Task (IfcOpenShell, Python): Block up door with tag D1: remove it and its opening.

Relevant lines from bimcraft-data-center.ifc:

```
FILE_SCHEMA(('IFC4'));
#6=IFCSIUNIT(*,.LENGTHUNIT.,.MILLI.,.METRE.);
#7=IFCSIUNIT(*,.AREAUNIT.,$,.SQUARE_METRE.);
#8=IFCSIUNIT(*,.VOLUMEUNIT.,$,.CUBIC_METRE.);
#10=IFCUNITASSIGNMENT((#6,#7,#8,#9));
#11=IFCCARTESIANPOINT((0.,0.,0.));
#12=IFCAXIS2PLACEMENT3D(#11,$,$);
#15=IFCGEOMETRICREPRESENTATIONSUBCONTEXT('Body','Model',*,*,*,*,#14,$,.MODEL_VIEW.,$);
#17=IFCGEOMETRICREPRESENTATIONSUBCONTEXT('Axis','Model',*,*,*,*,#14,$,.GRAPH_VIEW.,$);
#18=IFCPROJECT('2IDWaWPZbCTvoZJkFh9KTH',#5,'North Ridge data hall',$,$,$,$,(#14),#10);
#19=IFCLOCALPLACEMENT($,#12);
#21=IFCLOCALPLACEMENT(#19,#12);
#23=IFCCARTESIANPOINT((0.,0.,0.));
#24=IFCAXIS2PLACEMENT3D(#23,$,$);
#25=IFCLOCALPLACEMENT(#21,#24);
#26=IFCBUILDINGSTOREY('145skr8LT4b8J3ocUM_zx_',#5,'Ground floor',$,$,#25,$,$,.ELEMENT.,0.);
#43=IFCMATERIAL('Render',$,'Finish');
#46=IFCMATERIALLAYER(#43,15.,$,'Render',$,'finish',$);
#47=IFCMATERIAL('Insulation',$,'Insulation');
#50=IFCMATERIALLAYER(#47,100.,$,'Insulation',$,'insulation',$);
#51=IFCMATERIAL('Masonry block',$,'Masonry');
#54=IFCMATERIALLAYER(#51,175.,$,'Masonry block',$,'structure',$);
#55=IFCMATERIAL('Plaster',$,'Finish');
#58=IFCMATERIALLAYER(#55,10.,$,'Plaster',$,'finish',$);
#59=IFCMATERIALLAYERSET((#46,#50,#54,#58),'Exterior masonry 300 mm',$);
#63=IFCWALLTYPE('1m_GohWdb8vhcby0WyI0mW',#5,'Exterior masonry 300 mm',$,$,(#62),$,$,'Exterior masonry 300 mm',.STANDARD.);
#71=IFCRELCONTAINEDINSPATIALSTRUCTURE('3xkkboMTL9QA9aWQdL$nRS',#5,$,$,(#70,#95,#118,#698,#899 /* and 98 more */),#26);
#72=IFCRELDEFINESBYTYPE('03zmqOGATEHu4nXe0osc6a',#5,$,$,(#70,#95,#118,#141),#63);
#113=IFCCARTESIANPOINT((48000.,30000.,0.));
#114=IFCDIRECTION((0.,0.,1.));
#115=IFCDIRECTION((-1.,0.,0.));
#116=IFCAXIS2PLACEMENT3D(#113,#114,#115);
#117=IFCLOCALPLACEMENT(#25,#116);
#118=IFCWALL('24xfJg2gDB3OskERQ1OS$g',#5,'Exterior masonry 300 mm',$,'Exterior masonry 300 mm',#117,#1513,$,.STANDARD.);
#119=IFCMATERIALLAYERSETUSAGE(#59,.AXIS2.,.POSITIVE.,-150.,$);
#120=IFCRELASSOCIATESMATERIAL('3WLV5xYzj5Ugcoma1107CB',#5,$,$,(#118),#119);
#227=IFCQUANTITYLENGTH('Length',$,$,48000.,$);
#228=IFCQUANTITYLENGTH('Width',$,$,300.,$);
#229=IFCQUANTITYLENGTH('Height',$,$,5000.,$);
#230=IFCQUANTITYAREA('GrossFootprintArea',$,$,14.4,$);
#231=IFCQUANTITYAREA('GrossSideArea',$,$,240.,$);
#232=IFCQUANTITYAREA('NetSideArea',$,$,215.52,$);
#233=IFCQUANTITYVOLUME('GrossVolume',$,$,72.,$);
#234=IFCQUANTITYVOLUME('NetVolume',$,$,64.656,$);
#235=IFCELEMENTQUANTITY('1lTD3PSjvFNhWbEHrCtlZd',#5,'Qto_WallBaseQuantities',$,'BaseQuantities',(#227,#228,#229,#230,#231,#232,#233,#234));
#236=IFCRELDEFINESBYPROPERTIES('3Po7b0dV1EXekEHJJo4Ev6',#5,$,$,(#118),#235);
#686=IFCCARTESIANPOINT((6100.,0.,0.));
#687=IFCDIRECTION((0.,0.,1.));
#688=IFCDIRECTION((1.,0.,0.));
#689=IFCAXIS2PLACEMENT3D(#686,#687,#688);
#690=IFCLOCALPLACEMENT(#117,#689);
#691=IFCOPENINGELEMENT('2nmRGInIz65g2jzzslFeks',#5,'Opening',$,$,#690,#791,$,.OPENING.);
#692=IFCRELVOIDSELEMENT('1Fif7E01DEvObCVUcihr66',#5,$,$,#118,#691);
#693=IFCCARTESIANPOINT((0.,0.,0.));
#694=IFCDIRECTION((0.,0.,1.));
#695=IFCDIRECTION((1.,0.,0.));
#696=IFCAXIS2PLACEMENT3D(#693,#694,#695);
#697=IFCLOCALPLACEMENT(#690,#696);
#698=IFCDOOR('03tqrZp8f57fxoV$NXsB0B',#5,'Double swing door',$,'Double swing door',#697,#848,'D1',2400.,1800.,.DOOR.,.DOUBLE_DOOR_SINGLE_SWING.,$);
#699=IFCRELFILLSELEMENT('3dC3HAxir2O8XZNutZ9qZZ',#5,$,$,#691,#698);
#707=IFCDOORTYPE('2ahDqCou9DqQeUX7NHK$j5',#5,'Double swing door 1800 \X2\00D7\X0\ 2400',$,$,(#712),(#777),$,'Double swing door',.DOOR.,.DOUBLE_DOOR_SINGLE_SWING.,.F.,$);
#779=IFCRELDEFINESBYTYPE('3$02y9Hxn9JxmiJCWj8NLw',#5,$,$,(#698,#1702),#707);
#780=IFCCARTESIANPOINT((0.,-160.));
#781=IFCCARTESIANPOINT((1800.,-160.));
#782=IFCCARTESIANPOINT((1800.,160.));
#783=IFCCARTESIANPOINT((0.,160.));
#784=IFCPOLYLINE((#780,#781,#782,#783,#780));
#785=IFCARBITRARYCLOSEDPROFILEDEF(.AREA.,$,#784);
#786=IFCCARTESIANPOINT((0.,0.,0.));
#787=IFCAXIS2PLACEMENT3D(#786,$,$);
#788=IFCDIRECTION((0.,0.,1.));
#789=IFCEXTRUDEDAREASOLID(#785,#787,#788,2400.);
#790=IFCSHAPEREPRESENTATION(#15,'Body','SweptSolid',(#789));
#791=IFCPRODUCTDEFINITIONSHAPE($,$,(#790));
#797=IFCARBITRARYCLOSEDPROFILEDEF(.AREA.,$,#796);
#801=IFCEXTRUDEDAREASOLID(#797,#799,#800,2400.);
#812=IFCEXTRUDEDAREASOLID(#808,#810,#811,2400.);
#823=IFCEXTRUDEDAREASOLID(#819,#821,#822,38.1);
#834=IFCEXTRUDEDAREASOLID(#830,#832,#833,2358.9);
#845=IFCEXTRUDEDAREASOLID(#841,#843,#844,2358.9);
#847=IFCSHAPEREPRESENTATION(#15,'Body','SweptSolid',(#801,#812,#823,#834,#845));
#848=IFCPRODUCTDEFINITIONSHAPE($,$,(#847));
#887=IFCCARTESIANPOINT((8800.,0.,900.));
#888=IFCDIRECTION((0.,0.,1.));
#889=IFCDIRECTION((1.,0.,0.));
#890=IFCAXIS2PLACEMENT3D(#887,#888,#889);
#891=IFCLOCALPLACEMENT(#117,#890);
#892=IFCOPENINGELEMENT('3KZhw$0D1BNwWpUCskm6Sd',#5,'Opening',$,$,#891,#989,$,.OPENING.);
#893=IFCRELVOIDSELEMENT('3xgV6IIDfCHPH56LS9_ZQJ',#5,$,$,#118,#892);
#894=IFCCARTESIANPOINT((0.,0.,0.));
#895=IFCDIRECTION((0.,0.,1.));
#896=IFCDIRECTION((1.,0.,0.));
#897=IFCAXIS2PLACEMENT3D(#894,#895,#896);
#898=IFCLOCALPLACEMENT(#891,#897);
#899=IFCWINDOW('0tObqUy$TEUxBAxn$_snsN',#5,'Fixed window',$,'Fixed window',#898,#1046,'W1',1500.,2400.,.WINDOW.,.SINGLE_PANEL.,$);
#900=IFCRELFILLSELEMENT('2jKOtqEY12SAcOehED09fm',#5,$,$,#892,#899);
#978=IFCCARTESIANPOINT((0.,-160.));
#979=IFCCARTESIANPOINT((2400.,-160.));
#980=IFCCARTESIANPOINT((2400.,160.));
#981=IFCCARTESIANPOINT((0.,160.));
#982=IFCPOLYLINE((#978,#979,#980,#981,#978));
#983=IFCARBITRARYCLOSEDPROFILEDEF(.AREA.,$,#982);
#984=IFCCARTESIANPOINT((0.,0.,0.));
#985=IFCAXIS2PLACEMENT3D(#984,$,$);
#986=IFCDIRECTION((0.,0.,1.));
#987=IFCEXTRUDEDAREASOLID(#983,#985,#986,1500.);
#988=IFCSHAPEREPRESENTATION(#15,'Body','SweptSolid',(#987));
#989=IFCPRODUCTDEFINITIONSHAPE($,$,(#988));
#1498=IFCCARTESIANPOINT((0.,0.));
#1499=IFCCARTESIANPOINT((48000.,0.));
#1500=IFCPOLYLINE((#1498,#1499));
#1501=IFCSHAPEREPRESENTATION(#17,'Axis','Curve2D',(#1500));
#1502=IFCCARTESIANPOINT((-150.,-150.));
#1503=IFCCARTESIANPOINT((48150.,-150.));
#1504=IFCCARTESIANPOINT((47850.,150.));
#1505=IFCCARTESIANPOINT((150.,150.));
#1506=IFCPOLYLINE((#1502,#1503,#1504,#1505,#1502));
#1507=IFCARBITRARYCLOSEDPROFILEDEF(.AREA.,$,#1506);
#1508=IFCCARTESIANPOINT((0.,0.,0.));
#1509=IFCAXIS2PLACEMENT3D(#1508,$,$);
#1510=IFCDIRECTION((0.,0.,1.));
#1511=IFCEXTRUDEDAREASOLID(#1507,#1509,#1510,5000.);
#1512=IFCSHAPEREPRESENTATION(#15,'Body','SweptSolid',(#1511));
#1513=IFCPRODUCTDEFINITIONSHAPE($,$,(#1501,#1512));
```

```python
import ifcopenshell
import ifcopenshell.api.feature
import ifcopenshell.api.pset
import ifcopenshell.api.root
import ifcopenshell.geom
import ifcopenshell.util.element
import ifcopenshell.util.shape
import ifcopenshell.util.unit

model = ifcopenshell.open("bimcraft-data-center.ifc")
area_scale = ifcopenshell.util.unit.calculate_unit_scale(model, "AREAUNIT")
volume_scale = ifcopenshell.util.unit.calculate_unit_scale(model, "VOLUMEUNIT")
settings = ifcopenshell.geom.settings()


def volume(element):
    """Net volume in cubic metres, openings subtracted."""
    shape = ifcopenshell.geom.create_shape(settings, element)
    return ifcopenshell.util.shape.get_volume(shape.geometry)


door = model.by_guid("03tqrZp8f57fxoV$NXsB0B")
opening = door.FillsVoids[0].RelatingOpeningElement
wall = opening.VoidsElements[0].RelatingBuildingElement
before = volume(wall)

ifcopenshell.api.root.remove_product(model, product=door)
ifcopenshell.api.feature.remove_feature(model, feature=opening)

after = volume(wall)
thickness = 0.3  # wall thickness in metres

# Update the wall's stored quantities.
qto = model.by_id(ifcopenshell.util.element.get_pset(wall, "Qto_WallBaseQuantities", should_inherit=False)["id"])
ifcopenshell.api.pset.edit_qto(model, qto=qto, properties={
    "NetSideArea": after / thickness / area_scale,
    "NetVolume": after / volume_scale,
})

print(f"wall volume {before:.3f} -> {after:.3f} m3")

model.write("bimcraft-data-center_rev.ifc")
```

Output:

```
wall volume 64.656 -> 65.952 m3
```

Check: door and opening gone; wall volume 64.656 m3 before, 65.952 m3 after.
